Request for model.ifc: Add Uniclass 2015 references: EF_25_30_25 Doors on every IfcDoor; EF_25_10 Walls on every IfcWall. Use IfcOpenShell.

First a look at what the model holds.

```python
import ifcopenshell

model = ifcopenshell.open("model.ifc")
print(model.schema)
print("classifications:", [c.Name for c in model.by_type("IfcClassification")])
for ifc_class in ("IfcDoor", "IfcRoof", "IfcStair", "IfcWall", "IfcWindow"):
    print(ifc_class, len(model.by_type(ifc_class)))
```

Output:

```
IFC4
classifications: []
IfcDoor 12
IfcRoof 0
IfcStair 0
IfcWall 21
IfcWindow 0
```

```python
import ifcopenshell
import ifcopenshell.api.classification

model = ifcopenshell.open("model.ifc")

system = ifcopenshell.api.classification.add_classification(model, classification="Uniclass 2015")

codes = {
    "IfcDoor": ("EF_25_30_25", "Doors"),
    "IfcWall": ("EF_25_10", "Walls"),
}
for ifc_class, (code, name) in codes.items():
    products = model.by_type(ifc_class)
    ifcopenshell.api.classification.add_reference(
        model, products=products, classification=system, identification=code, name=name
    )
    print(code, len(products))

model.write("model_updated.ifc")
```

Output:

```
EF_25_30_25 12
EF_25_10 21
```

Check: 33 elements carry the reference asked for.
